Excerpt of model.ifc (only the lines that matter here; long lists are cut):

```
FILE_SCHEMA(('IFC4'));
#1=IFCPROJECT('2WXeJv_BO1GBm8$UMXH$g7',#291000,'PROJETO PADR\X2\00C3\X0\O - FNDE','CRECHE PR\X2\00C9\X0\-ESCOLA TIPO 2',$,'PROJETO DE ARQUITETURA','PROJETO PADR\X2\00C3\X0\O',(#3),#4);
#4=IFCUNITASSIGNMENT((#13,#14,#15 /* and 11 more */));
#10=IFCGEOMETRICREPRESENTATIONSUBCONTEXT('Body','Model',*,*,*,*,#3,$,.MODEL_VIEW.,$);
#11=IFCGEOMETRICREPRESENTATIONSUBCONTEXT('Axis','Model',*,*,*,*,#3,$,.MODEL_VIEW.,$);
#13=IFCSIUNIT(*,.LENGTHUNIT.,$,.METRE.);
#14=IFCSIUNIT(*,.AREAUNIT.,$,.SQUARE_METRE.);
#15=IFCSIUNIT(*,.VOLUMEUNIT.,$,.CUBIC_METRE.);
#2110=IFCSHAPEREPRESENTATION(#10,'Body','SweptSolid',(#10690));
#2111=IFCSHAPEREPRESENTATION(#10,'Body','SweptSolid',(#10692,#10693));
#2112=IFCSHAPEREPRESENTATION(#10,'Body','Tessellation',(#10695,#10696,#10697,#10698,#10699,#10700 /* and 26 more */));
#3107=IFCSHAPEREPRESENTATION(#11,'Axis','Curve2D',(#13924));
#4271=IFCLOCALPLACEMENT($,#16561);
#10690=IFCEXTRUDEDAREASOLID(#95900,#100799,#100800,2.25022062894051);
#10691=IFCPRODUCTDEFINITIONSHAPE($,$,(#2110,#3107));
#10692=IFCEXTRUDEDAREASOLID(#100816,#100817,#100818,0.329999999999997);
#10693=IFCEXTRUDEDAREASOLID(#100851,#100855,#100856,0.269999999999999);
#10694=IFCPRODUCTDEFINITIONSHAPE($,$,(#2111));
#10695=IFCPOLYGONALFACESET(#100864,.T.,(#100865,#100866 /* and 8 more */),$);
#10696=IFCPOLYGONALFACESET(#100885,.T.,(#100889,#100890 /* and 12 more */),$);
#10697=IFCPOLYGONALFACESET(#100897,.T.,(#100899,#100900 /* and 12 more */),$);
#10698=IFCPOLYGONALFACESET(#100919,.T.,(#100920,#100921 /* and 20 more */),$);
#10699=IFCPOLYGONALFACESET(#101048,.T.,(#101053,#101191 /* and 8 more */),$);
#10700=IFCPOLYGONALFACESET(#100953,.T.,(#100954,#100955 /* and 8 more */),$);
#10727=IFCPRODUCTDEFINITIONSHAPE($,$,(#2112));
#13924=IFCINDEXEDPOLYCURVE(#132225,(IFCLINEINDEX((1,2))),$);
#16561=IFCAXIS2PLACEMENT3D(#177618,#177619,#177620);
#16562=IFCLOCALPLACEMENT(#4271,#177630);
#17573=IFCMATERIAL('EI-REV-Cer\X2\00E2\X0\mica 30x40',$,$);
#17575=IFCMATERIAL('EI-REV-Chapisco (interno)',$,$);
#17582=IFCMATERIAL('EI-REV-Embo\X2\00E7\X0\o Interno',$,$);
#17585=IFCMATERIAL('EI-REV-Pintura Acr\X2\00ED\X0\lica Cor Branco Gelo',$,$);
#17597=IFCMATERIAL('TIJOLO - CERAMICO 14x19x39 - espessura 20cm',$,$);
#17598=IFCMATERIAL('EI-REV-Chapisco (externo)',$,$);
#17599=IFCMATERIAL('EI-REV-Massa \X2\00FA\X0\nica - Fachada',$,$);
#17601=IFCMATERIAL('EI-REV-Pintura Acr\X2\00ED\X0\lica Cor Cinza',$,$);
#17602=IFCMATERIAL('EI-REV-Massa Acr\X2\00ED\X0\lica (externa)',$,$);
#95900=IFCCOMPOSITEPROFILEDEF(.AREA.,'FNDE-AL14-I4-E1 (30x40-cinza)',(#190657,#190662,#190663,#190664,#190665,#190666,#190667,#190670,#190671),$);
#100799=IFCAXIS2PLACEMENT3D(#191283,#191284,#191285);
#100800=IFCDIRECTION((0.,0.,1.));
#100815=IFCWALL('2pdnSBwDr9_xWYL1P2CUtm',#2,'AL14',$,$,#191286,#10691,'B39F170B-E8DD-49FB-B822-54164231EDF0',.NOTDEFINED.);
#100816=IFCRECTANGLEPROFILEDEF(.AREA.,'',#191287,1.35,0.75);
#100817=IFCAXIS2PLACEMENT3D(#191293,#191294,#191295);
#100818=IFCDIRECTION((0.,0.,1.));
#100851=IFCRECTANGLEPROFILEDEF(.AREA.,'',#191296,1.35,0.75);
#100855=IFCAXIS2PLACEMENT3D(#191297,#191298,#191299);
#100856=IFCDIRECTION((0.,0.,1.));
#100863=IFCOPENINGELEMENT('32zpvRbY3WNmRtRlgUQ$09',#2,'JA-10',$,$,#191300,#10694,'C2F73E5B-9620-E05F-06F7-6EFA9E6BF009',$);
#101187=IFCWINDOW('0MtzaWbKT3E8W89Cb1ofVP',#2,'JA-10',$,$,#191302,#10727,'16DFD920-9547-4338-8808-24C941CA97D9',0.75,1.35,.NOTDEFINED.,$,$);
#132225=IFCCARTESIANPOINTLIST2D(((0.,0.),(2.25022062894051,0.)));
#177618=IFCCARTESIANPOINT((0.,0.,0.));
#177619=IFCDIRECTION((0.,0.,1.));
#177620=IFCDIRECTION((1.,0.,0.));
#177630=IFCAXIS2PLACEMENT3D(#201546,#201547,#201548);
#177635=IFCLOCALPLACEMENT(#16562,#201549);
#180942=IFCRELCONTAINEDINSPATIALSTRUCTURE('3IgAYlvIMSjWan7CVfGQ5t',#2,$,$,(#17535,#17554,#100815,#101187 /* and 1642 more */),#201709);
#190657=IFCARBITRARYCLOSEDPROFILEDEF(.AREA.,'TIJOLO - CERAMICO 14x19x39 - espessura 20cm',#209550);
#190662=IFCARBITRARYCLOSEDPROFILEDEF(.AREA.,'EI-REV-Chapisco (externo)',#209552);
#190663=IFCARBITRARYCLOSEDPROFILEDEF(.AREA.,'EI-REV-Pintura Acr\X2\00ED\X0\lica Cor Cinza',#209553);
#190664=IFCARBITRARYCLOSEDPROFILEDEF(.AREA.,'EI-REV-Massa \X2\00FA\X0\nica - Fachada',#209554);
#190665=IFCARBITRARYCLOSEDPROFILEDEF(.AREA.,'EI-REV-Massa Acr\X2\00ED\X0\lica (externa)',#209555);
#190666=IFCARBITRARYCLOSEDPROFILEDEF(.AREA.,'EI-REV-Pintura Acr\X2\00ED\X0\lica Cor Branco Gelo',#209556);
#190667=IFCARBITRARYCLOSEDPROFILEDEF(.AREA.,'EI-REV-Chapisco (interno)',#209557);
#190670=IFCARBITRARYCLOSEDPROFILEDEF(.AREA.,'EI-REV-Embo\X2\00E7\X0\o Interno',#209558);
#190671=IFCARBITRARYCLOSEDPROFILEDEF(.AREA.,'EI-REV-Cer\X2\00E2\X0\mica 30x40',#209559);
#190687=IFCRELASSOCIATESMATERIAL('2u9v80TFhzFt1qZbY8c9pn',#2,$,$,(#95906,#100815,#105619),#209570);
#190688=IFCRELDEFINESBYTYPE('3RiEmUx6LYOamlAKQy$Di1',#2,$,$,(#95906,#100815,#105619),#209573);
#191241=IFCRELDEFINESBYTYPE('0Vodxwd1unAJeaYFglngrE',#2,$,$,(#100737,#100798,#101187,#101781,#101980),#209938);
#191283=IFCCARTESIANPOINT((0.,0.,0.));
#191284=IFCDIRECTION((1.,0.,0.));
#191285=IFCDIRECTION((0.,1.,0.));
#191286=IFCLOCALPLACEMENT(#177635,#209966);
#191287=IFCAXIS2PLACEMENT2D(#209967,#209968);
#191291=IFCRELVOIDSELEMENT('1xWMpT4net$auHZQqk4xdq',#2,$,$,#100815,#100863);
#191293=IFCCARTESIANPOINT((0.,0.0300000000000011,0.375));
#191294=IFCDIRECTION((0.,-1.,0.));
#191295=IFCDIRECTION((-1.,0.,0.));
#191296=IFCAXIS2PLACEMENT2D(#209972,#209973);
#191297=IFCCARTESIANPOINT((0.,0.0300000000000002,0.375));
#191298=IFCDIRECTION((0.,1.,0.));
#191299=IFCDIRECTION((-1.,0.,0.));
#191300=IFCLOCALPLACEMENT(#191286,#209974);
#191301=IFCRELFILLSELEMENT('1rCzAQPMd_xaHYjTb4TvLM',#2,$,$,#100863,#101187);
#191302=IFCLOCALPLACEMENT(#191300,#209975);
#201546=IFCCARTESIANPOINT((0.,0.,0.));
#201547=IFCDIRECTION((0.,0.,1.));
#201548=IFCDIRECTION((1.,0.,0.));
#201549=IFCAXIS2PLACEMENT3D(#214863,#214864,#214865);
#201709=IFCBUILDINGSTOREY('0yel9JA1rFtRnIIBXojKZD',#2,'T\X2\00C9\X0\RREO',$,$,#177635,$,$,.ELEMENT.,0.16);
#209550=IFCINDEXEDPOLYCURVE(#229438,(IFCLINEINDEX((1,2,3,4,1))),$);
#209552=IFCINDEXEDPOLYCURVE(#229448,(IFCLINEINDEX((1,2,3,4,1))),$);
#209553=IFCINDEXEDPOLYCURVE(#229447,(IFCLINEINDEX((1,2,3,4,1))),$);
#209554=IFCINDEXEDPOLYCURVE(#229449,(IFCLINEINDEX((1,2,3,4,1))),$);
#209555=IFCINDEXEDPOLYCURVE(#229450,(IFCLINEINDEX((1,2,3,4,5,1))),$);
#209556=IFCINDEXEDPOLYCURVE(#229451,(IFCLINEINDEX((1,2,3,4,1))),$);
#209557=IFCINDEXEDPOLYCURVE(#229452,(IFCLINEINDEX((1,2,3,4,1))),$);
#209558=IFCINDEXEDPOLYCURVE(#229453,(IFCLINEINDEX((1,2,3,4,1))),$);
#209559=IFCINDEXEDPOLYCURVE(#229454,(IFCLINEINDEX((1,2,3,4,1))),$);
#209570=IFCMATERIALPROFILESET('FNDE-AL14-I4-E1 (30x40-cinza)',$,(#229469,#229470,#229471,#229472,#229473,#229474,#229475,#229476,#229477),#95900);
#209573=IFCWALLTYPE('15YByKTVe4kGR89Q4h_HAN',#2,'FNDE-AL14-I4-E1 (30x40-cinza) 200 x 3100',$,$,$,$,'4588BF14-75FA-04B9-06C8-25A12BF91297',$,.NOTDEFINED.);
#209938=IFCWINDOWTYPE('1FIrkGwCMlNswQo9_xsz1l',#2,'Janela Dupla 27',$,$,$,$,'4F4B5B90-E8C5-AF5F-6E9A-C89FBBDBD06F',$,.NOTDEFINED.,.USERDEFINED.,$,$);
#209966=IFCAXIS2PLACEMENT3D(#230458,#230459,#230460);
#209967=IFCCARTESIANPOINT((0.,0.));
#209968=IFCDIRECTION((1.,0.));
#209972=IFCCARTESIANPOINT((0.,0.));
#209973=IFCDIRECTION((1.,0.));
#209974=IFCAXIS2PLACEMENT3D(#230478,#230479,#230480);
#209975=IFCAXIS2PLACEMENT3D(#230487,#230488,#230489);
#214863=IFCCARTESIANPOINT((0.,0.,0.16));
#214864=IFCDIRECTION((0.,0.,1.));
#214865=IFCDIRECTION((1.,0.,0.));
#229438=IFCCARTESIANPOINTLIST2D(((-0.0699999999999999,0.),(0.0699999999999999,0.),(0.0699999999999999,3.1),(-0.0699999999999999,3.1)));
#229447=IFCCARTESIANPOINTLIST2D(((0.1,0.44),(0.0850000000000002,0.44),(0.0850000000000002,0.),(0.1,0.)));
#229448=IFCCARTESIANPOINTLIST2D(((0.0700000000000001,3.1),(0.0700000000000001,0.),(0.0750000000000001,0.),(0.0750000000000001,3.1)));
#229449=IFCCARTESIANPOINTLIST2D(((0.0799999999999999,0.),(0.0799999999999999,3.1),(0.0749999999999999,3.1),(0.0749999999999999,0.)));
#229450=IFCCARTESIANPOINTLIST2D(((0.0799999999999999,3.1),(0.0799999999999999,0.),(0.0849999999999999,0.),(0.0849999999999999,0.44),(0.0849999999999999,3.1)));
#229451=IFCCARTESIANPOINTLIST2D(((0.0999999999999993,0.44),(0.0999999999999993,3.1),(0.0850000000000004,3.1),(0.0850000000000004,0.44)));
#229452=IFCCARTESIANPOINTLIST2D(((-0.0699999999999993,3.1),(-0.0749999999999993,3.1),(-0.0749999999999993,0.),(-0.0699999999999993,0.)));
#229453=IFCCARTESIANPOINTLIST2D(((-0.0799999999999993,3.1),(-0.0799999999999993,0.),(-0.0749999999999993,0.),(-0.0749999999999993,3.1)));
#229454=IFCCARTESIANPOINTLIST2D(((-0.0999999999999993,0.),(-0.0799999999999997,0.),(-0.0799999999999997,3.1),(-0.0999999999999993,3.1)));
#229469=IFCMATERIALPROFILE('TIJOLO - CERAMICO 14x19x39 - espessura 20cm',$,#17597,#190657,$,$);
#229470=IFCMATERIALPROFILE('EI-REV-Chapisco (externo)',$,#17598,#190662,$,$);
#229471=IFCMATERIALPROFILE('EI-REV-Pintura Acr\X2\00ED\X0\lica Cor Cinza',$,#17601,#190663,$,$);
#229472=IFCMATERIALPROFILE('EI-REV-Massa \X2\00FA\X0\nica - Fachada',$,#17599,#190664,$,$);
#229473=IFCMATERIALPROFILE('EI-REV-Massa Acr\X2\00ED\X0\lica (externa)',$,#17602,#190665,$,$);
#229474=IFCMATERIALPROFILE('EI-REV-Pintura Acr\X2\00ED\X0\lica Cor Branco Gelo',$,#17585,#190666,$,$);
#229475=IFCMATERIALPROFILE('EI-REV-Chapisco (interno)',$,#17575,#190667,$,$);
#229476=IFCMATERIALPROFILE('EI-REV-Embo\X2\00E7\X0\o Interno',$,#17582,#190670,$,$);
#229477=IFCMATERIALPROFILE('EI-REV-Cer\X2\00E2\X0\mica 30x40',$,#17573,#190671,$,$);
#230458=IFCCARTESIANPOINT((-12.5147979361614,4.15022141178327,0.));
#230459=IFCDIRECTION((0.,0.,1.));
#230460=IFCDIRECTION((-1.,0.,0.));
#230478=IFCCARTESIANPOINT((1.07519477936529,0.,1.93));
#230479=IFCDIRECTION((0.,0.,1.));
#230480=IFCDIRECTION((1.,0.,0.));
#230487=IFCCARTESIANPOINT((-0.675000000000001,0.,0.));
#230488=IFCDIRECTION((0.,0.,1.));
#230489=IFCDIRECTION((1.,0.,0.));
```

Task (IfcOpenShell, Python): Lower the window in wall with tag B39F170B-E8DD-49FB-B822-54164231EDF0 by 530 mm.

```python
import numpy as np
import ifcopenshell
import ifcopenshell.api.geometry
import ifcopenshell.util.placement
import ifcopenshell.util.unit

model = ifcopenshell.open("model.ifc")
unit_scale = ifcopenshell.util.unit.calculate_unit_scale(model)

window = model.by_guid("0MtzaWbKT3E8W89Cb1ofVP")
opening = window.FillsVoids[0].RelatingOpeningElement
dz = -0.53

shift = np.array([0.0, 0.0, dz])
# The window is placed relative to its opening, so it follows when the opening moves.
matrix = ifcopenshell.util.placement.get_local_placement(opening.ObjectPlacement)
matrix[:3, 3] += shift
ifcopenshell.api.geometry.edit_object_placement(
    model, product=opening, matrix=matrix, is_si=False, should_transform_children=True
)

print(f"moved by {dz * unit_scale:+.3f} m")

model.write("model_v2.ifc")
```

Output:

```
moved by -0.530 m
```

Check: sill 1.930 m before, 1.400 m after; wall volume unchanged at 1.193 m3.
